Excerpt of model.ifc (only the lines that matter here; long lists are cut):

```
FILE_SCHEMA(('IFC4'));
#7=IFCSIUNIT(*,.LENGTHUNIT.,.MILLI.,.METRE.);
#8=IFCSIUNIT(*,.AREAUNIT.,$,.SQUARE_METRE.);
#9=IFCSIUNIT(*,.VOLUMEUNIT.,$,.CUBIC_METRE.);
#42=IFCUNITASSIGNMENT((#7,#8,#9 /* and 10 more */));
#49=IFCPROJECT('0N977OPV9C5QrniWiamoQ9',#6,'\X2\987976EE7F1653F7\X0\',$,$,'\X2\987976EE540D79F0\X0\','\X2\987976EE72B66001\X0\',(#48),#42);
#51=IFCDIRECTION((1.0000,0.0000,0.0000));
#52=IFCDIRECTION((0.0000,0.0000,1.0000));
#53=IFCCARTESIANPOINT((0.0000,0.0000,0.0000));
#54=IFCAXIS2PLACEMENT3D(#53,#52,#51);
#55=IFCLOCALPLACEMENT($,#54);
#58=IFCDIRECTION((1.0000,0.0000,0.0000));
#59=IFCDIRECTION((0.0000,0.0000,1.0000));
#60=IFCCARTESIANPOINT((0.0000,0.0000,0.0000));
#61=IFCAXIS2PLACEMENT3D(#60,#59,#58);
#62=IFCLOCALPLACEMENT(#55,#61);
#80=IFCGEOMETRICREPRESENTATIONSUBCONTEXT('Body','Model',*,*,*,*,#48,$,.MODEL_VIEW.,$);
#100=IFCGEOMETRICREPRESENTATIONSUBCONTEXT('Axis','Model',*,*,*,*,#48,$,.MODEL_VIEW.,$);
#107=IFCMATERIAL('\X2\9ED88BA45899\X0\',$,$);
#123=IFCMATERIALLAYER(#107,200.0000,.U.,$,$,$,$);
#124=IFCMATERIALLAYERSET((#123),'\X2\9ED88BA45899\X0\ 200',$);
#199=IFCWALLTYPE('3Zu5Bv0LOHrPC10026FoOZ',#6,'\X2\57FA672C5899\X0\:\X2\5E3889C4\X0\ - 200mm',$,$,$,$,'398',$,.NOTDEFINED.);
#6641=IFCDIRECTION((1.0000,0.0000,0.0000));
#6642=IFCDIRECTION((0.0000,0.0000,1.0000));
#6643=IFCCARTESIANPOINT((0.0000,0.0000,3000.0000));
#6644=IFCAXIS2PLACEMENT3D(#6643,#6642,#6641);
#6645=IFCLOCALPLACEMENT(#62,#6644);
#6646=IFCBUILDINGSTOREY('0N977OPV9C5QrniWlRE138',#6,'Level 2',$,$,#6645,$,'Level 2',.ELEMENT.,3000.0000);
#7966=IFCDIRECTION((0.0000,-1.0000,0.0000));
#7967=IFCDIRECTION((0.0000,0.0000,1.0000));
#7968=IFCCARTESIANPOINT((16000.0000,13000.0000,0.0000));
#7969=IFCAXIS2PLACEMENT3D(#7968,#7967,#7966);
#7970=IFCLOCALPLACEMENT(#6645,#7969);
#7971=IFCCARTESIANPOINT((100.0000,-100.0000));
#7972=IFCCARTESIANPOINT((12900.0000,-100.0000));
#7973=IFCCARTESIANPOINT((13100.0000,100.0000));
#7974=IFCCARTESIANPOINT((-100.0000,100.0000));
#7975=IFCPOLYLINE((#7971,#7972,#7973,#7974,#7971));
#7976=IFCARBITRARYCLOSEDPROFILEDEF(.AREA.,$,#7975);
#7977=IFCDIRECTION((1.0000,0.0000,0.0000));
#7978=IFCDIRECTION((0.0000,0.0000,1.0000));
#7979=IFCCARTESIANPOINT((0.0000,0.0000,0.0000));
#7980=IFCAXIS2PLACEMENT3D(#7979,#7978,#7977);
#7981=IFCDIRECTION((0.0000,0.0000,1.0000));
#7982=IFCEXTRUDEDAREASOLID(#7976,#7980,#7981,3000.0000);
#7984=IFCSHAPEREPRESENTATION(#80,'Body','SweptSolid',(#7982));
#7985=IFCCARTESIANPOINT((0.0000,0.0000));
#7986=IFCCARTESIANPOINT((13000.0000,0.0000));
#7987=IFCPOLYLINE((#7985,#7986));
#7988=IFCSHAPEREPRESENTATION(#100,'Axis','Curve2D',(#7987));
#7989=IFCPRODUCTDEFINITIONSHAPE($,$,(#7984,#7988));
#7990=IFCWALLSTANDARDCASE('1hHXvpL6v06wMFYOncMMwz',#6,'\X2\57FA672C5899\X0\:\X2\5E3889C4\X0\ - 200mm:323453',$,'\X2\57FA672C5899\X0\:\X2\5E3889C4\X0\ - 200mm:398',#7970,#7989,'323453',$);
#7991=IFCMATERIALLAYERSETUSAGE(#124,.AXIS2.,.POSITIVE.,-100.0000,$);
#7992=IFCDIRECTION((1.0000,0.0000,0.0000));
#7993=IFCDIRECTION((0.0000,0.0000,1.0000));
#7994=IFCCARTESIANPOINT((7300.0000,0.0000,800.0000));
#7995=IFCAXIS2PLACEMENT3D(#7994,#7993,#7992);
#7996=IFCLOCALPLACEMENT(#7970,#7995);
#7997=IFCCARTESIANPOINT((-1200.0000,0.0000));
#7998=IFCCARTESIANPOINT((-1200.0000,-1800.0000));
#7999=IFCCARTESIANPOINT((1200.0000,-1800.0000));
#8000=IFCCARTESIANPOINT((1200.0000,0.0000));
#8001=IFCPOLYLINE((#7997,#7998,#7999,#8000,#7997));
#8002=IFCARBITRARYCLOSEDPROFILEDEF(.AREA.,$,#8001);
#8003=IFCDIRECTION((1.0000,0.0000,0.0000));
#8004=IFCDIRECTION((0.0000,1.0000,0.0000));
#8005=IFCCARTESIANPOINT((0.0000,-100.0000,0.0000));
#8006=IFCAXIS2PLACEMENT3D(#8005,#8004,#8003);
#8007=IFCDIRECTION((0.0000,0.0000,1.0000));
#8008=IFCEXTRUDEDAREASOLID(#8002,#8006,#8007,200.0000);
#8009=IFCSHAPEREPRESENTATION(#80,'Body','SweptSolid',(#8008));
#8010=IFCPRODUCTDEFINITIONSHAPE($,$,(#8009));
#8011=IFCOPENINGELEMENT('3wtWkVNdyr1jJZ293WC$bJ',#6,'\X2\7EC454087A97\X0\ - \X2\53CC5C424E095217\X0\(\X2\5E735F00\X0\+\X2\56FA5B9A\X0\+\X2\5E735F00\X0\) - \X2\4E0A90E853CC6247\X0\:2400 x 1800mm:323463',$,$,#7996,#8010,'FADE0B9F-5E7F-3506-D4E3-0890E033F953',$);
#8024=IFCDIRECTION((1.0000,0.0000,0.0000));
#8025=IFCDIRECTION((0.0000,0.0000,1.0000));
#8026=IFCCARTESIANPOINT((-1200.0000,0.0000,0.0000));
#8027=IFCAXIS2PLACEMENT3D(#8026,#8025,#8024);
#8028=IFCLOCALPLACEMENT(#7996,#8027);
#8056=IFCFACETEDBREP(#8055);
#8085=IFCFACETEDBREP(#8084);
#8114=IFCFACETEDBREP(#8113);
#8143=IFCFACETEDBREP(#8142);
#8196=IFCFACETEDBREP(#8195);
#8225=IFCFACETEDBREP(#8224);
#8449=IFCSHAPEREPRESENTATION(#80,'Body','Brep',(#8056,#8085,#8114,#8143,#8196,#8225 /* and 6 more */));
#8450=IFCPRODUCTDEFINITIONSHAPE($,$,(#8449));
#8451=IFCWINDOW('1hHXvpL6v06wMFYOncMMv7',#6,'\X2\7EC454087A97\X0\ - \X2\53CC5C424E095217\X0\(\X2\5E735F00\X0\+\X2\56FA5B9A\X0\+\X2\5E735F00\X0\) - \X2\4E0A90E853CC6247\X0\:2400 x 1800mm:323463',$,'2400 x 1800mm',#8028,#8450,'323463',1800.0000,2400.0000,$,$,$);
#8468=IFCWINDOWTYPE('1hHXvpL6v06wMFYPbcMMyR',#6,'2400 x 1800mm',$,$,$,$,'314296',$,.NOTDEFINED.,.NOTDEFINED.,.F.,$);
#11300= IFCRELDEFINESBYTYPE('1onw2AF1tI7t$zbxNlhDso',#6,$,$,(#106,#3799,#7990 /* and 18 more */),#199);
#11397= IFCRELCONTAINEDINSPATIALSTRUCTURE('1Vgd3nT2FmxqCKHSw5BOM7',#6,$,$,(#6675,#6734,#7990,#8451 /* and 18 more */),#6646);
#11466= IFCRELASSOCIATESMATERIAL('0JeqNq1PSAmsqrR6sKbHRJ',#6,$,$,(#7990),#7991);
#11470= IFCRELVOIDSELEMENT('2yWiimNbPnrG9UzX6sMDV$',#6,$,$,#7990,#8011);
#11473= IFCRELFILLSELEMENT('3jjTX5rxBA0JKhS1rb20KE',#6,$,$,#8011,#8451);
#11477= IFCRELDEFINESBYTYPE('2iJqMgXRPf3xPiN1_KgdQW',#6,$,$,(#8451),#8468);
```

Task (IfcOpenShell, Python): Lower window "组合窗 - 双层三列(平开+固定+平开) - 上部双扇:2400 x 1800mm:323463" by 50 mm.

```python
import numpy as np
import ifcopenshell
import ifcopenshell.api.geometry
import ifcopenshell.util.placement
import ifcopenshell.util.unit

model = ifcopenshell.open("model.ifc")
unit_scale = ifcopenshell.util.unit.calculate_unit_scale(model)

window = model.by_id(8451)
opening = window.FillsVoids[0].RelatingOpeningElement
dz = -50.0

shift = np.array([0.0, 0.0, dz])
# The window is placed relative to its opening, so it follows when the opening moves.
matrix = ifcopenshell.util.placement.get_local_placement(opening.ObjectPlacement)
matrix[:3, 3] += shift
ifcopenshell.api.geometry.edit_object_placement(
    model, product=opening, matrix=matrix, is_si=False, should_transform_children=True
)

print(f"moved by {dz * unit_scale:+.3f} m")

model.write("model_edited.ifc")
```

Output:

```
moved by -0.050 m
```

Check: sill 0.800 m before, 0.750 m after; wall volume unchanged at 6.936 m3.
